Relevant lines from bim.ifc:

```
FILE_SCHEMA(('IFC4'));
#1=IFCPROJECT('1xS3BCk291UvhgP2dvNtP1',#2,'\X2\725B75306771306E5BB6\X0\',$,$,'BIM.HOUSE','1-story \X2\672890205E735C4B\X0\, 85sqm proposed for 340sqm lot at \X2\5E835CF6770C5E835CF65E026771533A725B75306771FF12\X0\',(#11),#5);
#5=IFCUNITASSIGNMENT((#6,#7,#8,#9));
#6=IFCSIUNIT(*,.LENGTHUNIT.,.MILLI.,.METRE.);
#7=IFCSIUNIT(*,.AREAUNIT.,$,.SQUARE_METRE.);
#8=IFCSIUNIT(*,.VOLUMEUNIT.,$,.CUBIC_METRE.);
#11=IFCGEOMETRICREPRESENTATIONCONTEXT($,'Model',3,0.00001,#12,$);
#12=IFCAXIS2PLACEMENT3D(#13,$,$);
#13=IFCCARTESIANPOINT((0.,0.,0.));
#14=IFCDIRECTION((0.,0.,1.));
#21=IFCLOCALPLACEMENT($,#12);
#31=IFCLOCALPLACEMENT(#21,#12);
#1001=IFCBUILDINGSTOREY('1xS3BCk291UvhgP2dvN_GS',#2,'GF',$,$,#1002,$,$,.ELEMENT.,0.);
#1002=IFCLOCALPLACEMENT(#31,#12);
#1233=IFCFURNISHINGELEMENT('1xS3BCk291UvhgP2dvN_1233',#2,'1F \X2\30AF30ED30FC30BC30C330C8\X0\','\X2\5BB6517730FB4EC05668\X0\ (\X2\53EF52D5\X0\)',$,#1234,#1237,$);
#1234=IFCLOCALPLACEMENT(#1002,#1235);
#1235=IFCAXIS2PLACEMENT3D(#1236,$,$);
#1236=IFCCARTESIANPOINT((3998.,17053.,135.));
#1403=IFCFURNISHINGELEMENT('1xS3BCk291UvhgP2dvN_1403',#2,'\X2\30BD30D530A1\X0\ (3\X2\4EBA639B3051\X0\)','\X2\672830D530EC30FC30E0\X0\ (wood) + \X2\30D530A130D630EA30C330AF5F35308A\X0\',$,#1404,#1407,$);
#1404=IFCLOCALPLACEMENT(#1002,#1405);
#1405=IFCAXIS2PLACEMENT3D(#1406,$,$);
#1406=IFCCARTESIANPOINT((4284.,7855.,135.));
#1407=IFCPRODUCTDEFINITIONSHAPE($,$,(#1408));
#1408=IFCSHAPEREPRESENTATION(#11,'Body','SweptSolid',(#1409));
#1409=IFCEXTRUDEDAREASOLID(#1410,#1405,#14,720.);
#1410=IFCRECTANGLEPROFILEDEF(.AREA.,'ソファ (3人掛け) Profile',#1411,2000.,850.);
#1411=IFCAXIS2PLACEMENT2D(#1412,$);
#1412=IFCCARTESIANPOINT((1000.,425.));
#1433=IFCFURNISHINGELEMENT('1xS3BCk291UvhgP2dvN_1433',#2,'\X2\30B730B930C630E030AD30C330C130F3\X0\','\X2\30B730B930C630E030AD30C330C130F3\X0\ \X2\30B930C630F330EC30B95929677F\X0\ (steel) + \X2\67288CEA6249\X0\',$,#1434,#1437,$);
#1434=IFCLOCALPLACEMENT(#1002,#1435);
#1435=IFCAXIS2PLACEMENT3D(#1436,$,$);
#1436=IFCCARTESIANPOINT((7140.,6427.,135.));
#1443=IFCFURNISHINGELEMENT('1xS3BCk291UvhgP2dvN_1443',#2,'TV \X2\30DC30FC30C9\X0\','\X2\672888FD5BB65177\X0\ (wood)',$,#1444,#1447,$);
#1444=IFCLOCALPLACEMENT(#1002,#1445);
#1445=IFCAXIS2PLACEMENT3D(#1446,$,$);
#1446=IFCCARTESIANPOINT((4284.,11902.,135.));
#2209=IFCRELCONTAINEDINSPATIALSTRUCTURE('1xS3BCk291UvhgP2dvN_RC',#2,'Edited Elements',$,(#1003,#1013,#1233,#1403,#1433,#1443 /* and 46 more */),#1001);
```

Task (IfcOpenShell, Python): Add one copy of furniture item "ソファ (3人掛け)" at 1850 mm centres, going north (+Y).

```python
import numpy as np
import ifcopenshell
import ifcopenshell.api.geometry
import ifcopenshell.api.root
import ifcopenshell.util.element
import ifcopenshell.util.placement

model = ifcopenshell.open("bim.ifc")


def reuse_history(source, copy):
    """copy_class also copies each property set's owner history, people and application; keep the originals."""
    for rel in copy.IsDefinedBy:
        if rel.is_a("IfcRelDefinesByProperties") and (history := rel.RelatingPropertyDefinition.OwnerHistory):
            rel.RelatingPropertyDefinition.OwnerHistory = source.OwnerHistory
            ifcopenshell.util.element.remove_deep2(model, history)


source = model.by_guid("1xS3BCk291UvhgP2dvN_1403")
base = ifcopenshell.util.placement.get_local_placement(source.ObjectPlacement)
step = np.array([0.0, 1.0, 0.0]) * 1850.0

for i in range(1, 2):
    copy = ifcopenshell.api.root.copy_class(model, product=source)
    copy.Representation = ifcopenshell.util.element.copy_deep(
        model, source.Representation, exclude=["IfcGeometricRepresentationContext", "IfcRepresentationMap"]
    )
    reuse_history(source, copy)
    matrix = base.copy()
    matrix[:3, 3] += i * step
    print("added at", matrix[:3, 3].round(3) + 0.0)
    ifcopenshell.api.geometry.edit_object_placement(model, product=copy, matrix=matrix, is_si=False)

model.write("bim_rev.ifc")
```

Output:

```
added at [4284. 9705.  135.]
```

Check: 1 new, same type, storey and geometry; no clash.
